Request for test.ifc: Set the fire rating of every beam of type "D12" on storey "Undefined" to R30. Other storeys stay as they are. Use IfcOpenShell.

First a look at what the model holds.

```python
import ifcopenshell
import ifcopenshell.util.element

model = ifcopenshell.open("test.ifc")
print(model.schema)
storey = next(s for s in model.by_type("IfcBuildingStorey") if s.Name == "Undefined")
beams = [e for e in ifcopenshell.util.element.get_decomposition(storey) if e.is_a("IfcBeam")]
seen = {}
for e in beams:
    element_type = ifcopenshell.util.element.get_type(e)
    key = (element_type.Name if element_type != e and element_type else None, ifcopenshell.util.element.get_pset(e, "Pset_BeamCommon", "FireRating"))
    seen[key] = seen.get(key, 0) + 1
for (name, value), count in sorted(seen.items(), key=str):
    print(count, "x", name, "|", value)
```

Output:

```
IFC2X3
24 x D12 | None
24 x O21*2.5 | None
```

```python
import ifcopenshell
import ifcopenshell.api.pset
import ifcopenshell.util.element

model = ifcopenshell.open("test.ifc")

storey = next(s for s in model.by_type("IfcBuildingStorey") if s.Name == "Undefined")
beams = [e for e in ifcopenshell.util.element.get_decomposition(storey) if e.is_a("IfcBeam")]

count = 0
for e in beams:
    element_type = ifcopenshell.util.element.get_type(e)
    if element_type in (None, e) or element_type.Name != "D12":
        continue
    found = ifcopenshell.util.element.get_pset(e, "Pset_BeamCommon", should_inherit=False)
    if found:
        pset = model.by_id(found["id"])
        if len(ifcopenshell.util.element.get_elements_by_pset(pset)) > 1:
            pset = ifcopenshell.api.pset.unshare_pset(model, products=[e], pset=pset)[0]
    else:
        pset = ifcopenshell.api.pset.add_pset(model, product=e, name="Pset_BeamCommon")
    ifcopenshell.api.pset.edit_pset(model, pset=pset, properties={"FireRating": "R30"})
    count += 1

print(count, "beams updated")

model.write("test_rev.ifc")
```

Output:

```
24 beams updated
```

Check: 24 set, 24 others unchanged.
